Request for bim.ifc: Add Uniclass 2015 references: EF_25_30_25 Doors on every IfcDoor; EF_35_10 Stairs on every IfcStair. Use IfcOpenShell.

First a look at what the model holds.

```python
import ifcopenshell

model = ifcopenshell.open("bim.ifc")
print(model.schema)
print("classifications:", [c.Name for c in model.by_type("IfcClassification")])
for ifc_class in ("IfcDoor", "IfcRoof", "IfcStair", "IfcWall", "IfcWindow"):
    print(ifc_class, len(model.by_type(ifc_class)))
```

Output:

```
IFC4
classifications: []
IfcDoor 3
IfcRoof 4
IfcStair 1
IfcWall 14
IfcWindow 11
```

```python
import ifcopenshell
import ifcopenshell.api.classification

model = ifcopenshell.open("bim.ifc")

system = ifcopenshell.api.classification.add_classification(model, classification="Uniclass 2015")

codes = {
    "IfcDoor": ("EF_25_30_25", "Doors"),
    "IfcStair": ("EF_35_10", "Stairs"),
}
for ifc_class, (code, name) in codes.items():
    products = model.by_type(ifc_class)
    ifcopenshell.api.classification.add_reference(
        model, products=products, classification=system, identification=code, name=name
    )
    print(code, len(products))

model.write("bim_v2.ifc")
```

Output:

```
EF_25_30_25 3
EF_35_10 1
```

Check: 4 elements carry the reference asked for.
